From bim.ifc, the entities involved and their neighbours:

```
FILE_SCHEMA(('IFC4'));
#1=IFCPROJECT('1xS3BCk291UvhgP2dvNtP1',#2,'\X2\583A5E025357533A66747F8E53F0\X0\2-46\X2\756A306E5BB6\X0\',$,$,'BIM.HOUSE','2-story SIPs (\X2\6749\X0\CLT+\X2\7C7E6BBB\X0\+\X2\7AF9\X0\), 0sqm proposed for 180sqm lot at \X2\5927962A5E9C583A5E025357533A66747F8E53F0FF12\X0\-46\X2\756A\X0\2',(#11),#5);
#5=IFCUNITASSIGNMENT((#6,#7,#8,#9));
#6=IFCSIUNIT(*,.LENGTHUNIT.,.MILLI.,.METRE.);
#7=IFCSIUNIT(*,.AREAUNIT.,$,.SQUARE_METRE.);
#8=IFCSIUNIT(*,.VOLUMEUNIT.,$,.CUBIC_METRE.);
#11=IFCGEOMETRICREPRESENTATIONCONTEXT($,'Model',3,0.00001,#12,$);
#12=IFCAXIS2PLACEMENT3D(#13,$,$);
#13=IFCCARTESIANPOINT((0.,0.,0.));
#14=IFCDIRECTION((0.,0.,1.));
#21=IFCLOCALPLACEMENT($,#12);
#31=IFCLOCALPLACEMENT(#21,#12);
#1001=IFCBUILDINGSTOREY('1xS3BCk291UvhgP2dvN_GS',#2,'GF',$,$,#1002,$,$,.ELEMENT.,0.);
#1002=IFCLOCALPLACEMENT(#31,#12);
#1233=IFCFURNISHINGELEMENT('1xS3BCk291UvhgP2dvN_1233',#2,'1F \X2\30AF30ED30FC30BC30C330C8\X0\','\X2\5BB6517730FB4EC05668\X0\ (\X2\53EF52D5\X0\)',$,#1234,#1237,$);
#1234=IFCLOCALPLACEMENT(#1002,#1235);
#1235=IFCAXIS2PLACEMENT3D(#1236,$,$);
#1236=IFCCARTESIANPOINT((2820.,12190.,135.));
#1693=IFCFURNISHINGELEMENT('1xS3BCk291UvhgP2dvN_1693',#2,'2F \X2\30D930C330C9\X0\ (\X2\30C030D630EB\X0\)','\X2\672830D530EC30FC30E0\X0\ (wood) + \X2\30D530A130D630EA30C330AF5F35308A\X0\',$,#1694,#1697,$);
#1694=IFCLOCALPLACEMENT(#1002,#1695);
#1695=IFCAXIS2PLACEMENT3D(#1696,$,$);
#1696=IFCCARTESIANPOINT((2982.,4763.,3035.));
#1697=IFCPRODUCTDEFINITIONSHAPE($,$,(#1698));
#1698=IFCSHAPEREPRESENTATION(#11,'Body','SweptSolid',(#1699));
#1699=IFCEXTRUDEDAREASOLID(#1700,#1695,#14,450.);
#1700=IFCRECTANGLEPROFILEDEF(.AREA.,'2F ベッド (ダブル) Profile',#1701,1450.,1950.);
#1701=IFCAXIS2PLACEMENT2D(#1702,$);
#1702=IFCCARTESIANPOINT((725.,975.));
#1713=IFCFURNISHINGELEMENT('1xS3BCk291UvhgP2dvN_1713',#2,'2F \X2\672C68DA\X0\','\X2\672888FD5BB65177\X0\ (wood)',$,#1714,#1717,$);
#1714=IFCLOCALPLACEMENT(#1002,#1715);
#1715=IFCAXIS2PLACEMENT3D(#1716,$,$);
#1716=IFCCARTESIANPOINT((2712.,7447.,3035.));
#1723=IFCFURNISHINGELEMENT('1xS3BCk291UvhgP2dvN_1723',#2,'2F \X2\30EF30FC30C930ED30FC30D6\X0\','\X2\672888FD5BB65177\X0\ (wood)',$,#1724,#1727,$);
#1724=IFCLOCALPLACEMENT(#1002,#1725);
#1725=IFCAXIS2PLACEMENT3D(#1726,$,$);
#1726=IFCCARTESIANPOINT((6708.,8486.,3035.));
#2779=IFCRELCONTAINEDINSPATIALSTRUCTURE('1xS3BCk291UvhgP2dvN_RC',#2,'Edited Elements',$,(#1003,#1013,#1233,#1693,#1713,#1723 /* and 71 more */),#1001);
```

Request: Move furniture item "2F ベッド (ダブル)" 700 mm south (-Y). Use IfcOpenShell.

```python
import ifcopenshell
import ifcopenshell.api.geometry
import ifcopenshell.util.placement
import ifcopenshell.util.unit

model = ifcopenshell.open("bim.ifc")
unit_scale = ifcopenshell.util.unit.calculate_unit_scale(model)

item = model.by_guid("1xS3BCk291UvhgP2dvN_1693")
matrix = ifcopenshell.util.placement.get_local_placement(item.ObjectPlacement)
matrix[1, 3] -= 0.7 / unit_scale
ifcopenshell.api.geometry.edit_object_placement(model, product=item, matrix=matrix, is_si=False)

print(ifcopenshell.util.placement.get_local_placement(item.ObjectPlacement).round(3) + 0.0)

model.write("bim_v2.ifc")
```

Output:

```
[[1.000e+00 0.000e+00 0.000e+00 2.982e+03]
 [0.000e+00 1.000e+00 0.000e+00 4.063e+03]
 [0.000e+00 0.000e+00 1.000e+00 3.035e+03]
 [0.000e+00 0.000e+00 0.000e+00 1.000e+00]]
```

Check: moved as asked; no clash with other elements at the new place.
